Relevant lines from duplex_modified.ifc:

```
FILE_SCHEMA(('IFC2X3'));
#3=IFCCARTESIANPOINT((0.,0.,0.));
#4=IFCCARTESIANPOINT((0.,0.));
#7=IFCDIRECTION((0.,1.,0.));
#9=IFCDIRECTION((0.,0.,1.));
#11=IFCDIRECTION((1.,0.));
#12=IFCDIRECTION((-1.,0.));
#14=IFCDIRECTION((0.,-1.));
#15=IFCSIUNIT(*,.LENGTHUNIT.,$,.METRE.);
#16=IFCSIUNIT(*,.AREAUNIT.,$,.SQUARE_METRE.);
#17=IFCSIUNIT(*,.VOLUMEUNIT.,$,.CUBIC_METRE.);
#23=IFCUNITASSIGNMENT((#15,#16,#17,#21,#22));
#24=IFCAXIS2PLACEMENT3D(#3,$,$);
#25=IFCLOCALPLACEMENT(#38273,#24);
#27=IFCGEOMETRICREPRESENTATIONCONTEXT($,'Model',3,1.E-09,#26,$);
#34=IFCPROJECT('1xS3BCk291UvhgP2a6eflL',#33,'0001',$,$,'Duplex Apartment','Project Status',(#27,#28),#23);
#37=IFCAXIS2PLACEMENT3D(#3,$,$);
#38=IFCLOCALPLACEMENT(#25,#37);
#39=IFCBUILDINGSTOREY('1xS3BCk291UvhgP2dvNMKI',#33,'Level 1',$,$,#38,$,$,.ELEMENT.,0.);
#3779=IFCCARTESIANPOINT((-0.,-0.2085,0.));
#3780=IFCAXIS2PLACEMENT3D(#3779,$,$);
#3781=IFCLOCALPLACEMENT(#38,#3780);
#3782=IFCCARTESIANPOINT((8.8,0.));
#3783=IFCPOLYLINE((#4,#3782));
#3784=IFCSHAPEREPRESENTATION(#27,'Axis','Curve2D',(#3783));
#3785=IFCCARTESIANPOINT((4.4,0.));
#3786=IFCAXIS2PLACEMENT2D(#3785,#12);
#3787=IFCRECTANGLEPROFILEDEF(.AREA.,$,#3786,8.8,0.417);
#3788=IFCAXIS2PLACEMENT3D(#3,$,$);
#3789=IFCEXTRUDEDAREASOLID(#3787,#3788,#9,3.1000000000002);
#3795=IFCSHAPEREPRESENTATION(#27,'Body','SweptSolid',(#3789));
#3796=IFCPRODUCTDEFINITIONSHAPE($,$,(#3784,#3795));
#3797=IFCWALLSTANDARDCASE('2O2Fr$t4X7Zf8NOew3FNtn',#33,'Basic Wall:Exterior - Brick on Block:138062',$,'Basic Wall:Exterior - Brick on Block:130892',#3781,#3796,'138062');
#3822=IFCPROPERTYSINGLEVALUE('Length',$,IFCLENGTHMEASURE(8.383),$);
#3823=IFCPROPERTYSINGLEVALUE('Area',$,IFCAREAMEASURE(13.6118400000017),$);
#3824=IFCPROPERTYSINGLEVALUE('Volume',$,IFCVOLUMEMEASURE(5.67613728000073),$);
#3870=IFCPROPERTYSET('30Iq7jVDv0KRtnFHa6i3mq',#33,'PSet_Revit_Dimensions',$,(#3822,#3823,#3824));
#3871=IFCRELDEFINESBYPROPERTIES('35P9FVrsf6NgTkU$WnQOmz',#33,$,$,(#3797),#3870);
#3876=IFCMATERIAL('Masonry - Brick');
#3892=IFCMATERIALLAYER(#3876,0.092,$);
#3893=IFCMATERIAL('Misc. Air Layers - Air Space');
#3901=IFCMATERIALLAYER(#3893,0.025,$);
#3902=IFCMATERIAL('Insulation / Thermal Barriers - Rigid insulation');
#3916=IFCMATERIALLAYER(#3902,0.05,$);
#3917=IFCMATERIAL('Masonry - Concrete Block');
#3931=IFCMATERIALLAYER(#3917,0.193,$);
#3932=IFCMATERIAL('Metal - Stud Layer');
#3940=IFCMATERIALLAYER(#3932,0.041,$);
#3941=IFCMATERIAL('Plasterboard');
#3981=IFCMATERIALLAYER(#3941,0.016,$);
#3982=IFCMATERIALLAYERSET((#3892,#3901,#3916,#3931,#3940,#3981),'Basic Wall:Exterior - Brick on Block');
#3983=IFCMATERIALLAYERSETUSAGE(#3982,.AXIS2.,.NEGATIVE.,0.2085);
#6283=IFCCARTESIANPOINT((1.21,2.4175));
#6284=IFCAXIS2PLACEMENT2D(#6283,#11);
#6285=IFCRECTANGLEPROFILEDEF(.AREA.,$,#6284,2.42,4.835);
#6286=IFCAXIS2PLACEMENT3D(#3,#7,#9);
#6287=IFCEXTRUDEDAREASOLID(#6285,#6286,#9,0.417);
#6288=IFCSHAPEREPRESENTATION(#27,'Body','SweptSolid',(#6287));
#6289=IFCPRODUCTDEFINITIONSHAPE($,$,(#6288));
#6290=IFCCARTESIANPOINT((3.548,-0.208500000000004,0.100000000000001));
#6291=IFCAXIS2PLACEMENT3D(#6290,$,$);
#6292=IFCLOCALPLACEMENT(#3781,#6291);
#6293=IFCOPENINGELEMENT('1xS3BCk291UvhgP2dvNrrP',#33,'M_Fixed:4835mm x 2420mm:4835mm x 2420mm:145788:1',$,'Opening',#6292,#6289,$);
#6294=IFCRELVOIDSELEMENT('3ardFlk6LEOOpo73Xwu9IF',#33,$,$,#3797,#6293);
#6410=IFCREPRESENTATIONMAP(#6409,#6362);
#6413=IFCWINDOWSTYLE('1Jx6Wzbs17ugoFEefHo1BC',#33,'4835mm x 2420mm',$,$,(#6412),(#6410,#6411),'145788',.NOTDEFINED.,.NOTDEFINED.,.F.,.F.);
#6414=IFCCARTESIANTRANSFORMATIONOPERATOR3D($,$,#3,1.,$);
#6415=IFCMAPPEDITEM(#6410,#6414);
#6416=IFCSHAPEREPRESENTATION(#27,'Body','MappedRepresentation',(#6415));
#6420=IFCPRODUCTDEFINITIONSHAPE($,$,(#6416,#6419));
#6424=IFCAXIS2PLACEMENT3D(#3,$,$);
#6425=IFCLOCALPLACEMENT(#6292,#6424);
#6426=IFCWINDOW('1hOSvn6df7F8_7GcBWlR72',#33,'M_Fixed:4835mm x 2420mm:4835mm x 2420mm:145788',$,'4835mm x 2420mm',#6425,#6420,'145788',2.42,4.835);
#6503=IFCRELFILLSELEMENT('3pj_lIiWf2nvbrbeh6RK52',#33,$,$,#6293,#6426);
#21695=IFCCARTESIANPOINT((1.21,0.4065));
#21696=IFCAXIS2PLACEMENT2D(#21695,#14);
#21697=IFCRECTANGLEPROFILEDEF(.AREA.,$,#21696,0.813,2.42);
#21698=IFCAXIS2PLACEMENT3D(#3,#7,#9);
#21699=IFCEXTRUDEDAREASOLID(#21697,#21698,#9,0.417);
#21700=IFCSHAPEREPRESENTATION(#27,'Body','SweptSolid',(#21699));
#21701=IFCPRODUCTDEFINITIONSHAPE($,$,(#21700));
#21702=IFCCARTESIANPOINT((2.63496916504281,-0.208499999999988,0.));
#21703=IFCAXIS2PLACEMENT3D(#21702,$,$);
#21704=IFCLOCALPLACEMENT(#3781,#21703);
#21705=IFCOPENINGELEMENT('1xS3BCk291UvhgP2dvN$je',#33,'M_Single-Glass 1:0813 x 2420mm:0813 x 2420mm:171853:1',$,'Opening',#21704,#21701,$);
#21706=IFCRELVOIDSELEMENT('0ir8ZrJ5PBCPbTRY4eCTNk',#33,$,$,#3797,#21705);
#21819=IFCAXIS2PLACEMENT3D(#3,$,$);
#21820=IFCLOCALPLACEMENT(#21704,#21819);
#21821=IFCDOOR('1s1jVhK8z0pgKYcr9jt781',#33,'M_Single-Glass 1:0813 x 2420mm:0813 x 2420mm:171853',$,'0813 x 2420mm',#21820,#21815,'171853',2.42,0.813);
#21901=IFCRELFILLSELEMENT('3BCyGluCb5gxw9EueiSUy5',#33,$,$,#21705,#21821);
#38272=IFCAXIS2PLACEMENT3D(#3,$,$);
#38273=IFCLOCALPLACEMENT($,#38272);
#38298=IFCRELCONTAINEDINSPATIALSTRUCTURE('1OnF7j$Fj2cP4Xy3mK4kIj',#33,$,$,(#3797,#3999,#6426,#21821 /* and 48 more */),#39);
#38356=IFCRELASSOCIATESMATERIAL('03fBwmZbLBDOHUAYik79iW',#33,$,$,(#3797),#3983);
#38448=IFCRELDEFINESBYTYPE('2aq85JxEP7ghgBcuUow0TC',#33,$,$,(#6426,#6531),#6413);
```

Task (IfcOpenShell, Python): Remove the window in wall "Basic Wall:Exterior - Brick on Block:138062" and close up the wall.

```python
import ifcopenshell
import ifcopenshell.api.feature
import ifcopenshell.api.pset
import ifcopenshell.api.root
import ifcopenshell.geom
import ifcopenshell.util.element
import ifcopenshell.util.shape
import ifcopenshell.util.unit

model = ifcopenshell.open("duplex_modified.ifc")
area_scale = ifcopenshell.util.unit.calculate_unit_scale(model, "AREAUNIT")
volume_scale = ifcopenshell.util.unit.calculate_unit_scale(model, "VOLUMEUNIT")
settings = ifcopenshell.geom.settings()


def volume(element):
    """Net volume in cubic metres, openings subtracted."""
    shape = ifcopenshell.geom.create_shape(settings, element)
    return ifcopenshell.util.shape.get_volume(shape.geometry)


window = model.by_guid("1hOSvn6df7F8_7GcBWlR72")
opening = window.FillsVoids[0].RelatingOpeningElement
wall = opening.VoidsElements[0].RelatingBuildingElement
before = volume(wall)

ifcopenshell.api.root.remove_product(model, product=window)
ifcopenshell.api.feature.remove_feature(model, feature=opening)

after = volume(wall)
thickness = 0.417  # wall thickness in metres

# Update the wall's stored quantities.
pset = model.by_id(ifcopenshell.util.element.get_pset(wall, "PSet_Revit_Dimensions", should_inherit=False)["id"])
ifcopenshell.api.pset.edit_pset(model, pset=pset, properties={
    "Area": model.create_entity("IfcAreaMeasure", after / thickness / area_scale),
    "Volume": model.create_entity("IfcVolumeMeasure", after / volume_scale),
})

print(f"wall volume {before:.3f} -> {after:.3f} m3")

model.write("duplex_modified_rev.ifc")
```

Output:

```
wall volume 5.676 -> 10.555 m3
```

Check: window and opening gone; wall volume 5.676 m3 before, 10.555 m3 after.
